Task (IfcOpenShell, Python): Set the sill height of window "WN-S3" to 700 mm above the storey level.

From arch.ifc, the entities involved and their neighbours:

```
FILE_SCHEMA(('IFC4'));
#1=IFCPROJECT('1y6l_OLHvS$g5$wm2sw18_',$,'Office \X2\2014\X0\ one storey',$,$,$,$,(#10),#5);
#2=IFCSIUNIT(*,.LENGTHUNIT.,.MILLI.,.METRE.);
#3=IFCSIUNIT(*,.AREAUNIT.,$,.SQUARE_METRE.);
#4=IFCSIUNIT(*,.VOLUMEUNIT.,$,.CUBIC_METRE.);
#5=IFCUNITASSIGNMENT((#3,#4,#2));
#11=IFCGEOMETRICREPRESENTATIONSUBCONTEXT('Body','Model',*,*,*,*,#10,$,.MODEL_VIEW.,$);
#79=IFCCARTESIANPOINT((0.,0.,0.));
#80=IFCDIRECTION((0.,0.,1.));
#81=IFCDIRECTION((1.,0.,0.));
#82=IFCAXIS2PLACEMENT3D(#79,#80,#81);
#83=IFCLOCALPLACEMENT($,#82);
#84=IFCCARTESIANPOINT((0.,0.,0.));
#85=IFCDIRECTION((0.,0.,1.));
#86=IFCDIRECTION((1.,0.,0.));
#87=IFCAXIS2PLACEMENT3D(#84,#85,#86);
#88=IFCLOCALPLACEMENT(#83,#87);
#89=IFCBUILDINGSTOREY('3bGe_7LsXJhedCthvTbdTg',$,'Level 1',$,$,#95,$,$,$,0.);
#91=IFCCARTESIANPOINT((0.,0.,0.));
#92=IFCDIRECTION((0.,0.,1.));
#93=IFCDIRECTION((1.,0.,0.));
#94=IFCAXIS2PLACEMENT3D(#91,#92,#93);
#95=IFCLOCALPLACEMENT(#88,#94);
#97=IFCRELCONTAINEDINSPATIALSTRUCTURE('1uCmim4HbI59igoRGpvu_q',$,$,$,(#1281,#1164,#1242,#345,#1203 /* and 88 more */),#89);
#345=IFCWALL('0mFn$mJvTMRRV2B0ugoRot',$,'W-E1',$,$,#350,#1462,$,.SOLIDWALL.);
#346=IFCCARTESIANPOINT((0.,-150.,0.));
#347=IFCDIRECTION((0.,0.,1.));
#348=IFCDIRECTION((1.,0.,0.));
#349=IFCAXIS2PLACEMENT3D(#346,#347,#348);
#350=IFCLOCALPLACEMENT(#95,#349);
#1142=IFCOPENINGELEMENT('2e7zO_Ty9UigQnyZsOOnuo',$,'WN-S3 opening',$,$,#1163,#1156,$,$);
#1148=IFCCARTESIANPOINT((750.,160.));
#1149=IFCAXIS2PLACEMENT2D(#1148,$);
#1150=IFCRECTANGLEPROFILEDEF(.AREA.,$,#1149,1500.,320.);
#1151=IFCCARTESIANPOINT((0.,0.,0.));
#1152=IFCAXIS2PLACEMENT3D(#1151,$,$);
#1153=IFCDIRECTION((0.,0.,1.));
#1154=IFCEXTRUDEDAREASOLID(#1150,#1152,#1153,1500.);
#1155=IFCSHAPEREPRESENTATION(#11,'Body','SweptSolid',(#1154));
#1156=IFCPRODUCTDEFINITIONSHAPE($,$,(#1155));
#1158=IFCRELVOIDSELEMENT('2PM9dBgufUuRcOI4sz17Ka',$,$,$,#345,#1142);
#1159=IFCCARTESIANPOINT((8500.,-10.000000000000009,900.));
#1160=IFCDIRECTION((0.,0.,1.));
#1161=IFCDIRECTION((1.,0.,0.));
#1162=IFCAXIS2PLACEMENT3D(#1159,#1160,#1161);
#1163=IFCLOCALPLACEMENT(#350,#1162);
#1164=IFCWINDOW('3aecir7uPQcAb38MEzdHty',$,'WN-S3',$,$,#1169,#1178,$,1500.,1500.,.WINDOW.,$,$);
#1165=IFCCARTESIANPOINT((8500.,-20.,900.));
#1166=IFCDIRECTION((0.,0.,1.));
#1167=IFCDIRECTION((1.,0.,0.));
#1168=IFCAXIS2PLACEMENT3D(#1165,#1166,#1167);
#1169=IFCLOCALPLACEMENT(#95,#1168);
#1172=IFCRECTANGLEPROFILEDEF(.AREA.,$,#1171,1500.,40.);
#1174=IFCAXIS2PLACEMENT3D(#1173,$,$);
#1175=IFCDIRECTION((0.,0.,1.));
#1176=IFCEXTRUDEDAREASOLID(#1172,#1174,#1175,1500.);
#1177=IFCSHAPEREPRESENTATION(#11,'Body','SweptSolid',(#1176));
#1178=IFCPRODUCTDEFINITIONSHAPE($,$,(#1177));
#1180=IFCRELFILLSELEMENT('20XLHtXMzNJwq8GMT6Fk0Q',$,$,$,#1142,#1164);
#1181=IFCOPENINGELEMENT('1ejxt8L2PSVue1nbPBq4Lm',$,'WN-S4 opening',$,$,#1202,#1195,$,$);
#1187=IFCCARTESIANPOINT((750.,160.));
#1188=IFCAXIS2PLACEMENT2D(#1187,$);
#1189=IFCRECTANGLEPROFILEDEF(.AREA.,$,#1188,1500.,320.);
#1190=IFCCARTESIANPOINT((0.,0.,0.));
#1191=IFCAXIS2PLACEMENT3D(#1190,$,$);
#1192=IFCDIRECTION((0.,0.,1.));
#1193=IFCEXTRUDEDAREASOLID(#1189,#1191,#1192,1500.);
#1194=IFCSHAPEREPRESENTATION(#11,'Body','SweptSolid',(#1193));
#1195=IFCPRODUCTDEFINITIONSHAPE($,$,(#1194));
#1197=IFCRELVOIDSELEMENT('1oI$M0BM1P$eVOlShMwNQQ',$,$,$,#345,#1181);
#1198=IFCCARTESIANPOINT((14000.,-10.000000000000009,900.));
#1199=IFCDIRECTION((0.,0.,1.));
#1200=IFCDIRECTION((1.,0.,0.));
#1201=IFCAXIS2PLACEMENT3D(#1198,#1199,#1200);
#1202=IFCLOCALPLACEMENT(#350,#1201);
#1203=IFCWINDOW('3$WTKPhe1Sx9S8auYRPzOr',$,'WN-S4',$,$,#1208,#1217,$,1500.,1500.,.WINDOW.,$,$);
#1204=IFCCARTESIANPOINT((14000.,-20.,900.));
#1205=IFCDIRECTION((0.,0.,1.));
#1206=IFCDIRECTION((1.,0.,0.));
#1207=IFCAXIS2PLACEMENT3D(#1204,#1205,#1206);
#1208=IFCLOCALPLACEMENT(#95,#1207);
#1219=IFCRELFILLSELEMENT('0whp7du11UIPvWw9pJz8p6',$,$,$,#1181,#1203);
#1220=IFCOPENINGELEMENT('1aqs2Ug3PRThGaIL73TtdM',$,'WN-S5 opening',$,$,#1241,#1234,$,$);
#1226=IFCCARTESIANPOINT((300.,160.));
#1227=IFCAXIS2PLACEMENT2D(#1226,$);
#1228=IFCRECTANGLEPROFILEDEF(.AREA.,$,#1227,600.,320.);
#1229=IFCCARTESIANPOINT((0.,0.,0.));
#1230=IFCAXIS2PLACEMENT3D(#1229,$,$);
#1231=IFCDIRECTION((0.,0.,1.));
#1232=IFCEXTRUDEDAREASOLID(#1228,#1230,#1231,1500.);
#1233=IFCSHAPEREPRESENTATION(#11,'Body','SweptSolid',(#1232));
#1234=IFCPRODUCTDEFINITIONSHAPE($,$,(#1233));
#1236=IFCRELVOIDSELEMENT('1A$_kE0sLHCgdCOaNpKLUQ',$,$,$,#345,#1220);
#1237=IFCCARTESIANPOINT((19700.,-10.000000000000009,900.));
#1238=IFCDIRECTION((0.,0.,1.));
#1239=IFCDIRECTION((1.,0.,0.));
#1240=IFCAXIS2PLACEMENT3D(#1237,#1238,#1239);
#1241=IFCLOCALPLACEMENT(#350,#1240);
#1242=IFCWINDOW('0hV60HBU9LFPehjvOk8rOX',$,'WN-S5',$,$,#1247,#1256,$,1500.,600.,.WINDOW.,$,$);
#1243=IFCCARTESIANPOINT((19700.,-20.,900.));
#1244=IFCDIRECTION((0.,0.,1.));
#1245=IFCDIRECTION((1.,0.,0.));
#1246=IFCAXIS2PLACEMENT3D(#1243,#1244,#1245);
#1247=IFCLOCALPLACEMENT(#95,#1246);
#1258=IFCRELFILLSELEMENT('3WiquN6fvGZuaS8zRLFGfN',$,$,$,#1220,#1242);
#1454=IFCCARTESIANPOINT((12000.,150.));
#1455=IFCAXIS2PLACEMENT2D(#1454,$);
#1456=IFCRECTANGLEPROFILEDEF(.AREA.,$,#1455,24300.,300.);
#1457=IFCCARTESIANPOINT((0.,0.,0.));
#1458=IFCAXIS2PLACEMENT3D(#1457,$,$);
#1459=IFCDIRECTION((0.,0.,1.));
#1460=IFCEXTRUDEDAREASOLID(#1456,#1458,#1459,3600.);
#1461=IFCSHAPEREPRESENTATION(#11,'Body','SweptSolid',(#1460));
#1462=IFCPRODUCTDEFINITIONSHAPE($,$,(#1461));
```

```python
import numpy as np
import ifcopenshell
import ifcopenshell.api.geometry
import ifcopenshell.geom
import ifcopenshell.util.element
import ifcopenshell.util.placement
import ifcopenshell.util.shape
import ifcopenshell.util.unit

model = ifcopenshell.open("arch.ifc")
unit_scale = ifcopenshell.util.unit.calculate_unit_scale(model)

window = model.by_guid("3aecir7uPQcAb38MEzdHty")
opening = window.FillsVoids[0].RelatingOpeningElement
storey = ifcopenshell.util.element.get_container(window, ifc_class="IfcBuildingStorey")
level = ifcopenshell.util.placement.get_local_placement(storey.ObjectPlacement)[2, 3]

# The opening's origin need not be at the sill, so measure its lowest point.
shape = ifcopenshell.geom.create_shape(ifcopenshell.geom.settings(), opening)
bottom = ifcopenshell.util.shape.get_shape_bottom_elevation(shape, shape.geometry) / unit_scale
dz = level + 0.7 / unit_scale - bottom

shift = np.array([0.0, 0.0, dz])
# The window is not placed relative to its opening, so move both.
for product in (opening, window):
    matrix = ifcopenshell.util.placement.get_local_placement(product.ObjectPlacement)
    matrix[:3, 3] += shift
    ifcopenshell.api.geometry.edit_object_placement(model, product=product, matrix=matrix, is_si=False)

print(f"moved by {dz * unit_scale:+.3f} m")

model.write("arch-out.ifc")
```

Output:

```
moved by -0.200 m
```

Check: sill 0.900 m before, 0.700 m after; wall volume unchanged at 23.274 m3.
